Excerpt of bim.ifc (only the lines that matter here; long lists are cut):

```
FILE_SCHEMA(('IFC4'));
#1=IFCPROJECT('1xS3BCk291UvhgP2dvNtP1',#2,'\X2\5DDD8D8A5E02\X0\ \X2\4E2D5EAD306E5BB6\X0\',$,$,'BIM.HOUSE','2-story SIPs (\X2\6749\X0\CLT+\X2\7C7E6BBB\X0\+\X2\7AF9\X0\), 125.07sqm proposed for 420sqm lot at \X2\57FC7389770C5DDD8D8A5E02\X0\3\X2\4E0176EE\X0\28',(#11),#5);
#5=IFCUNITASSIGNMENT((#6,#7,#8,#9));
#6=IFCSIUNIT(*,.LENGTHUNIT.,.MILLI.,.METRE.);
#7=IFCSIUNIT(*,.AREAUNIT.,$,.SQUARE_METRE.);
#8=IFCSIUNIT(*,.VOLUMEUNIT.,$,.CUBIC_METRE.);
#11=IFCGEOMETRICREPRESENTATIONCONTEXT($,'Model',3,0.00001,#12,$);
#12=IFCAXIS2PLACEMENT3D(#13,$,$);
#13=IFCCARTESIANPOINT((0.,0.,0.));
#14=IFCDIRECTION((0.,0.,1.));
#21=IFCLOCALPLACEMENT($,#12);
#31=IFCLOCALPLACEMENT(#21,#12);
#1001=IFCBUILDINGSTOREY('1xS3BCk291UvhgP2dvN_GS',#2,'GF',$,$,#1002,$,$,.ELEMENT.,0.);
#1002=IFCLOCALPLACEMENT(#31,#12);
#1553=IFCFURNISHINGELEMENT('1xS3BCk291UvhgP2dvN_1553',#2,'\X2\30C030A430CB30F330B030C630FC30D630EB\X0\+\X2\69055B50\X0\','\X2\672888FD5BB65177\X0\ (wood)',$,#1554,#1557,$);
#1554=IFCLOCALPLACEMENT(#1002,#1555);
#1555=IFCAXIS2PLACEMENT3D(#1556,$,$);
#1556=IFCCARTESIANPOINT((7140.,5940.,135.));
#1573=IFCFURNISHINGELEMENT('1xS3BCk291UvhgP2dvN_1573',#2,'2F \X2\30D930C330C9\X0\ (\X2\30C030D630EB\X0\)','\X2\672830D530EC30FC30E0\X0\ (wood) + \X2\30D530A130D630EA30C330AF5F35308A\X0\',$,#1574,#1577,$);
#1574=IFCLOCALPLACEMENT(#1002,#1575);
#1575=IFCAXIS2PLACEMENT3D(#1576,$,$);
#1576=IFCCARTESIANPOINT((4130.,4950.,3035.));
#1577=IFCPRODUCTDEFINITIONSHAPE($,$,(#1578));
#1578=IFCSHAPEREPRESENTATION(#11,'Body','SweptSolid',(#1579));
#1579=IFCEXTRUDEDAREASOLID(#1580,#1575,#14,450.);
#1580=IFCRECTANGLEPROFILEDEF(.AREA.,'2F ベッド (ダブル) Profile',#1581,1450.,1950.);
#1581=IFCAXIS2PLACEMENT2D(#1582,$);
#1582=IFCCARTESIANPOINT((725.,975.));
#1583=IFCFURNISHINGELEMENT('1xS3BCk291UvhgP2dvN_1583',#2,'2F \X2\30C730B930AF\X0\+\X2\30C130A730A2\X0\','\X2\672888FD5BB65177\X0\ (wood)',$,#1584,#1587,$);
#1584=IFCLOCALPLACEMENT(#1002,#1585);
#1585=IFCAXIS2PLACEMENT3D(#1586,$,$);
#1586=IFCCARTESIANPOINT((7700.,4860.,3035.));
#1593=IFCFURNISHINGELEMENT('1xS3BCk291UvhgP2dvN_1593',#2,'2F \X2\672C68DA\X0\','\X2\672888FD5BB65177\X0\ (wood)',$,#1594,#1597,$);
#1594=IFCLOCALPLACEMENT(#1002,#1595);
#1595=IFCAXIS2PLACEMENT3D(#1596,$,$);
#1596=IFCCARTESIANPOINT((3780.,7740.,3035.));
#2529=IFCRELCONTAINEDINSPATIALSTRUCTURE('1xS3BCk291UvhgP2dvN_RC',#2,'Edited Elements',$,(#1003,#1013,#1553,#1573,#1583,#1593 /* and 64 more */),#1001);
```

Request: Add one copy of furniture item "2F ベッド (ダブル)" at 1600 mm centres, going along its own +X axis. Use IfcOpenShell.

```python
import ifcopenshell
import ifcopenshell.api.geometry
import ifcopenshell.api.root
import ifcopenshell.util.element
import ifcopenshell.util.placement
import ifcopenshell.util.unit

model = ifcopenshell.open("bim.ifc")
unit_scale = ifcopenshell.util.unit.calculate_unit_scale(model)


def reuse_history(source, copy):
    """copy_class also copies each property set's owner history, people and application; keep the originals."""
    for rel in copy.IsDefinedBy:
        if rel.is_a("IfcRelDefinesByProperties") and (history := rel.RelatingPropertyDefinition.OwnerHistory):
            rel.RelatingPropertyDefinition.OwnerHistory = source.OwnerHistory
            ifcopenshell.util.element.remove_deep2(model, history)


source = model.by_guid("1xS3BCk291UvhgP2dvN_1573")
base = ifcopenshell.util.placement.get_local_placement(source.ObjectPlacement)
step = base[:3, 0] * 1.6 / unit_scale

for i in range(1, 2):
    copy = ifcopenshell.api.root.copy_class(model, product=source)
    copy.Representation = ifcopenshell.util.element.copy_deep(
        model, source.Representation, exclude=["IfcGeometricRepresentationContext", "IfcRepresentationMap"]
    )
    reuse_history(source, copy)
    matrix = base.copy()
    matrix[:3, 3] += i * step
    print("added at", matrix[:3, 3].round(3) + 0.0)
    ifcopenshell.api.geometry.edit_object_placement(model, product=copy, matrix=matrix, is_si=False)

model.write("bim-out.ifc")
```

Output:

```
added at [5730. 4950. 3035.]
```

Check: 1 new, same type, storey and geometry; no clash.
